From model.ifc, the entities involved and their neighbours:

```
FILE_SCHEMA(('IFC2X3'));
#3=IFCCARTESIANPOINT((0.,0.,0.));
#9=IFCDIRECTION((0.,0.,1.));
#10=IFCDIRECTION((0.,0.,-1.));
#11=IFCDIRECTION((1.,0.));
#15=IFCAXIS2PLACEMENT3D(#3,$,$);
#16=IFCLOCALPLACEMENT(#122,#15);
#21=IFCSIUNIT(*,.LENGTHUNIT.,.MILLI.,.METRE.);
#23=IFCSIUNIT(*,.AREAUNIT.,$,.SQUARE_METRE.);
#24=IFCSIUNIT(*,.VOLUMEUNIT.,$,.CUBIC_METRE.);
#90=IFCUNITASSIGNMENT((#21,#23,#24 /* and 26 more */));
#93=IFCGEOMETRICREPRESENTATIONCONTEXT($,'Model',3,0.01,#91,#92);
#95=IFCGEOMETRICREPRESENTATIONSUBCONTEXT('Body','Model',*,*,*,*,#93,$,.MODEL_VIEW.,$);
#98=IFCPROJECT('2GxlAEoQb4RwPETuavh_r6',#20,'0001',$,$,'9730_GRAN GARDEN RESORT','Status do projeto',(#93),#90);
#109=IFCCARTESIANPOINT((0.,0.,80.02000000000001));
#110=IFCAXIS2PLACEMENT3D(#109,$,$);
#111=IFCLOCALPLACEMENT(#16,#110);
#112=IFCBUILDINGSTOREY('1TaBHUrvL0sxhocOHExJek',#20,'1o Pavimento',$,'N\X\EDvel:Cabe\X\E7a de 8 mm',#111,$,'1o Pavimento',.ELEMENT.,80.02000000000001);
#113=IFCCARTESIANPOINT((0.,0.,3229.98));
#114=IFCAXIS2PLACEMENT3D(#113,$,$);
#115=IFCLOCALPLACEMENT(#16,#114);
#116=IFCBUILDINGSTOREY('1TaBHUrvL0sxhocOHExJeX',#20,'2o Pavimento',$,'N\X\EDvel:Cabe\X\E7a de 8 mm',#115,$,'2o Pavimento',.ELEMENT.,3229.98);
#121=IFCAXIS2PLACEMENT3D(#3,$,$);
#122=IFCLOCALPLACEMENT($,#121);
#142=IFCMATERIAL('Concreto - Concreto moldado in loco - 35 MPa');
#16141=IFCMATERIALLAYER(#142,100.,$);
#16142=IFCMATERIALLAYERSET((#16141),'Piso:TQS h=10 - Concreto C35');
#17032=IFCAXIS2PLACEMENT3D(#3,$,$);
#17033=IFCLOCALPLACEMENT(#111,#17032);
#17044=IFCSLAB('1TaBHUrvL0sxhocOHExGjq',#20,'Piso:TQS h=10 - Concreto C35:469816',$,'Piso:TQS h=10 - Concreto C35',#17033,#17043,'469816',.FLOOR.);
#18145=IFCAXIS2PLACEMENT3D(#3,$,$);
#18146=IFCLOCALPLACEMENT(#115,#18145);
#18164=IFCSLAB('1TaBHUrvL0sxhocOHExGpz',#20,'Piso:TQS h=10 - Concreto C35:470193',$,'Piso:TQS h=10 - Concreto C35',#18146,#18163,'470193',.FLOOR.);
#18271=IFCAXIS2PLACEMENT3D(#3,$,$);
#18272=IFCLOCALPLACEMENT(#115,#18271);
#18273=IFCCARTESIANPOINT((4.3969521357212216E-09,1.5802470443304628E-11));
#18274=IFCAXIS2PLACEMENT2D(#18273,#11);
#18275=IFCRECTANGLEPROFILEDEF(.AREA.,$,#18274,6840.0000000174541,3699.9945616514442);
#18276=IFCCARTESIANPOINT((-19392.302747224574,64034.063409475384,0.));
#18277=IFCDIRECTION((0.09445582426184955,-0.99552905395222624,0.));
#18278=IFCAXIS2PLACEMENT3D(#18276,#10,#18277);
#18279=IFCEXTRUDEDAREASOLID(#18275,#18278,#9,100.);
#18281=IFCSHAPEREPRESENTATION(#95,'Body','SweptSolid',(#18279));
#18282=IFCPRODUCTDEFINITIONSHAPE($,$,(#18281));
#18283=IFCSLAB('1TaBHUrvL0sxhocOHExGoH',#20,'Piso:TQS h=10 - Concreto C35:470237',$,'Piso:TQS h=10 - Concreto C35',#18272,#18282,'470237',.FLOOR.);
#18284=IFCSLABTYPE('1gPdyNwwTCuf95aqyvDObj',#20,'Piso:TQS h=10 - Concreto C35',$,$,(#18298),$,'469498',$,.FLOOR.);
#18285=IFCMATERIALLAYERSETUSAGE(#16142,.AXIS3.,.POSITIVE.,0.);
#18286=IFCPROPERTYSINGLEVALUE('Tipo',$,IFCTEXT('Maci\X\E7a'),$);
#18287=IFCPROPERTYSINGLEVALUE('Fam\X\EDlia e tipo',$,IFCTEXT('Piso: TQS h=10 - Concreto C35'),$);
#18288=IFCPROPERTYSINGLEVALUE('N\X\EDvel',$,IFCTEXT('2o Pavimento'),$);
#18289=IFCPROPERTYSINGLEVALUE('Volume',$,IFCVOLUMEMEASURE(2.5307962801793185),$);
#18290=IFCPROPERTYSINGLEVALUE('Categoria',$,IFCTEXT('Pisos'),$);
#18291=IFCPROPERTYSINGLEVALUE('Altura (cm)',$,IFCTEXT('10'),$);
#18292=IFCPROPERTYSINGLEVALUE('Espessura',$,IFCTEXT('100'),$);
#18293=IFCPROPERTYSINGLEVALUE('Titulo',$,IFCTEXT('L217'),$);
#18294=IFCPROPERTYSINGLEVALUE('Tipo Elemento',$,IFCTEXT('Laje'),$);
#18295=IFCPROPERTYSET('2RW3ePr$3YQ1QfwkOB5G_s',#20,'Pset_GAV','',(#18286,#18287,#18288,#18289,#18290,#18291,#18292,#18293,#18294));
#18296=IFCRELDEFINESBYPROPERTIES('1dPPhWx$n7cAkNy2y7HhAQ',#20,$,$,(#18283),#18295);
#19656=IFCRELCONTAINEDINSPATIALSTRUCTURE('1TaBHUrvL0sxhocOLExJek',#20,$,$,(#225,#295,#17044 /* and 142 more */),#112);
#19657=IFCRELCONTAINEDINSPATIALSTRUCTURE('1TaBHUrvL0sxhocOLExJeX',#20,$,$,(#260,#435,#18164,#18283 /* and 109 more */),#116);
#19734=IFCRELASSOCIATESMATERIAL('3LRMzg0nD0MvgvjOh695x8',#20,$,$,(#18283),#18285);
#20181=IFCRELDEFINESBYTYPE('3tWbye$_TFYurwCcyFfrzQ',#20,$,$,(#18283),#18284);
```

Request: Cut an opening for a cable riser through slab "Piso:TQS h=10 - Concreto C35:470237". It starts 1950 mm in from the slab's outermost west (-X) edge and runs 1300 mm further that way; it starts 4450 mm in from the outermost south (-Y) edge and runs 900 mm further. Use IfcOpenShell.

```python
import numpy as np
import ifcopenshell
import ifcopenshell.api.feature
import ifcopenshell.api.geometry
import ifcopenshell.api.pset
import ifcopenshell.api.root
import ifcopenshell.geom
import ifcopenshell.util.element
import ifcopenshell.util.placement
import ifcopenshell.util.representation
import ifcopenshell.util.shape
import ifcopenshell.util.unit

model = ifcopenshell.open("model.ifc")
unit_scale = ifcopenshell.util.unit.calculate_unit_scale(model)
volume_scale = ifcopenshell.util.unit.calculate_unit_scale(model, "VOLUMEUNIT")
settings = ifcopenshell.geom.settings()


def volume(element):
    """Net volume in cubic metres, openings subtracted."""
    shape = ifcopenshell.geom.create_shape(settings, element)
    return ifcopenshell.util.shape.get_volume(shape.geometry)


slab = model.by_id(18283)
before = volume(slab)

# Extent in the slab's own axes, in metres. The edges named are its -X and -Y sides.
slab_shape = ifcopenshell.geom.create_shape(settings, slab)
vertices = ifcopenshell.util.shape.get_vertices(slab_shape.geometry)
x_min, y_min, bottom = vertices.min(axis=0)
top = vertices[:, 2].max()

opening = ifcopenshell.api.root.create_entity(model, ifc_class="IfcOpeningElement", name="Cable riser opening")
context = ifcopenshell.util.representation.get_context(model, "Model", "Body", "MODEL_VIEW")
width, depth = 1.3, 0.9
outline = [(0.0, 0.0), (width, 0.0), (width, depth), (0.0, depth), (0.0, 0.0)]
# Overshoot both faces by 50 mm so the cut is clean.
shape = ifcopenshell.api.geometry.add_slab_representation(
    model, context=context, depth=top - bottom + 0.1, polyline=outline
)
ifcopenshell.api.geometry.assign_representation(model, product=opening, representation=shape)

matrix = ifcopenshell.util.placement.get_local_placement(slab.ObjectPlacement)
matrix[:, 3] = matrix @ np.append(np.array([x_min + 1.95, y_min + 4.45, bottom - 0.05]) / unit_scale, 1.0)
ifcopenshell.api.geometry.edit_object_placement(model, product=opening, matrix=matrix, is_si=False)
ifcopenshell.api.feature.add_feature(model, feature=opening, element=slab)

after = volume(slab)

# Update the slab's stored quantities.
pset = model.by_id(ifcopenshell.util.element.get_pset(slab, "Pset_GAV", should_inherit=False)["id"])
ifcopenshell.api.pset.edit_pset(model, pset=pset, properties={
    "Volume": model.create_entity("IfcVolumeMeasure", after / volume_scale),
})

print(f"slab volume {before:.3f} -> {after:.3f} m3")

model.write("model_updated.ifc")
```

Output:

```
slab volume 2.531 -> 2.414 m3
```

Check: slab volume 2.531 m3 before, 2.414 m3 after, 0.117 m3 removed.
